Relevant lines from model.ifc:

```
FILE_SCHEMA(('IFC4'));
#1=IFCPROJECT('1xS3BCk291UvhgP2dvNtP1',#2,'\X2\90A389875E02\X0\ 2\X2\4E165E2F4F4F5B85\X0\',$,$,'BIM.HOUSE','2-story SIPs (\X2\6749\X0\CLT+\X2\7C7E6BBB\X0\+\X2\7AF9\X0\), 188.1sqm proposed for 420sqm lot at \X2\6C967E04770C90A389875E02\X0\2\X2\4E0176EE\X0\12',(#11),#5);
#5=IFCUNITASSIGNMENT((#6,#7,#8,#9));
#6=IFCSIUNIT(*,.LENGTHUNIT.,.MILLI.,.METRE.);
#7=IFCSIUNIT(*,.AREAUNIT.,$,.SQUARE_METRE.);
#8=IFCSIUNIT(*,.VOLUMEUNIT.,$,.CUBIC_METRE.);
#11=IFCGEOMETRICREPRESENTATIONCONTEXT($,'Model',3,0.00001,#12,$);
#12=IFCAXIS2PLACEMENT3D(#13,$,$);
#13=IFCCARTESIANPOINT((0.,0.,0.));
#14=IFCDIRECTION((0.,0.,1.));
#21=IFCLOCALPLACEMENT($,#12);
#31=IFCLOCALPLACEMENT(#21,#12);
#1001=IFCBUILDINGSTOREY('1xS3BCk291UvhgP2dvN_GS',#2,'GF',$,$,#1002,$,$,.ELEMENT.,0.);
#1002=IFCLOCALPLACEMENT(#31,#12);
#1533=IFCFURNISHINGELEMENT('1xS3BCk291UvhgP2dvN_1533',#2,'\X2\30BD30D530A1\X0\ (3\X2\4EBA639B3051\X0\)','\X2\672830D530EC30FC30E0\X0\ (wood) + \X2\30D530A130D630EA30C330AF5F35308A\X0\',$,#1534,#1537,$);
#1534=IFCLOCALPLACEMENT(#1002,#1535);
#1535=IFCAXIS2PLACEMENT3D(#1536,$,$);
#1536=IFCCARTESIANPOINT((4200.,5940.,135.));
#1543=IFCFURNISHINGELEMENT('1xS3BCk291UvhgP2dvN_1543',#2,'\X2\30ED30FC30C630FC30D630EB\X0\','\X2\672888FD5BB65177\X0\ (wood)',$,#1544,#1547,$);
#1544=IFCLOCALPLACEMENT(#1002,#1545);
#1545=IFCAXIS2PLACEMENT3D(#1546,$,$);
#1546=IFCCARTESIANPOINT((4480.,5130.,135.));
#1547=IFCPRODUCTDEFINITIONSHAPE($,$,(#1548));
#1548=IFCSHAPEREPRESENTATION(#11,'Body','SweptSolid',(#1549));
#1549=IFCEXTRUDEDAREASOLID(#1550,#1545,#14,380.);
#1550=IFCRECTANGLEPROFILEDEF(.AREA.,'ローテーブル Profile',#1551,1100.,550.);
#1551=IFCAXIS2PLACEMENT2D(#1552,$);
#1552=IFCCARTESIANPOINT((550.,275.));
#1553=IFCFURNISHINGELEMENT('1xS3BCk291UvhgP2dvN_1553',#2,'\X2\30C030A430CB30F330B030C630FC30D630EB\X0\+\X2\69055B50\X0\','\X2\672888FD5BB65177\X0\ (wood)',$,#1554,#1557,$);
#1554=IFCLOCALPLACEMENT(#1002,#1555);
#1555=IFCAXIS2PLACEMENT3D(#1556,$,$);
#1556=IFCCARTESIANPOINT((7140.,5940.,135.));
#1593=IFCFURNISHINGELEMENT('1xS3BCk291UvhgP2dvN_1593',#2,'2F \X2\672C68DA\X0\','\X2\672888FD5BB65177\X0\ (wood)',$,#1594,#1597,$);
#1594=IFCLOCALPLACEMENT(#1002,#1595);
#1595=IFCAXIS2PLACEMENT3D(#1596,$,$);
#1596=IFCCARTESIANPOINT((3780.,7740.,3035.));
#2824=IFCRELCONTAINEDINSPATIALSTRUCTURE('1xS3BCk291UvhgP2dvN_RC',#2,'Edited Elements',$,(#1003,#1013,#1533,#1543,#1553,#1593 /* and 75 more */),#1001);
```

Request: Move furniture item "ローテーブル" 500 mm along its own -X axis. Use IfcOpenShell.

```python
import ifcopenshell
import ifcopenshell.api.geometry
import ifcopenshell.util.placement

model = ifcopenshell.open("model.ifc")

item = model.by_guid("1xS3BCk291UvhgP2dvN_1543")
matrix = ifcopenshell.util.placement.get_local_placement(item.ObjectPlacement)
matrix[:3, 3] -= matrix[:3, 0] * 500.0
ifcopenshell.api.geometry.edit_object_placement(model, product=item, matrix=matrix, is_si=False)

print(ifcopenshell.util.placement.get_local_placement(item.ObjectPlacement).round(3) + 0.0)

model.write("model_rev.ifc")
```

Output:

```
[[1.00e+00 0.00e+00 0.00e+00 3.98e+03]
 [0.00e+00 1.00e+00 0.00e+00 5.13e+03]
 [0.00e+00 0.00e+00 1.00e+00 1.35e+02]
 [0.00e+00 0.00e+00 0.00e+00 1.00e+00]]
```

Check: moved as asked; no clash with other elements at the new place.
